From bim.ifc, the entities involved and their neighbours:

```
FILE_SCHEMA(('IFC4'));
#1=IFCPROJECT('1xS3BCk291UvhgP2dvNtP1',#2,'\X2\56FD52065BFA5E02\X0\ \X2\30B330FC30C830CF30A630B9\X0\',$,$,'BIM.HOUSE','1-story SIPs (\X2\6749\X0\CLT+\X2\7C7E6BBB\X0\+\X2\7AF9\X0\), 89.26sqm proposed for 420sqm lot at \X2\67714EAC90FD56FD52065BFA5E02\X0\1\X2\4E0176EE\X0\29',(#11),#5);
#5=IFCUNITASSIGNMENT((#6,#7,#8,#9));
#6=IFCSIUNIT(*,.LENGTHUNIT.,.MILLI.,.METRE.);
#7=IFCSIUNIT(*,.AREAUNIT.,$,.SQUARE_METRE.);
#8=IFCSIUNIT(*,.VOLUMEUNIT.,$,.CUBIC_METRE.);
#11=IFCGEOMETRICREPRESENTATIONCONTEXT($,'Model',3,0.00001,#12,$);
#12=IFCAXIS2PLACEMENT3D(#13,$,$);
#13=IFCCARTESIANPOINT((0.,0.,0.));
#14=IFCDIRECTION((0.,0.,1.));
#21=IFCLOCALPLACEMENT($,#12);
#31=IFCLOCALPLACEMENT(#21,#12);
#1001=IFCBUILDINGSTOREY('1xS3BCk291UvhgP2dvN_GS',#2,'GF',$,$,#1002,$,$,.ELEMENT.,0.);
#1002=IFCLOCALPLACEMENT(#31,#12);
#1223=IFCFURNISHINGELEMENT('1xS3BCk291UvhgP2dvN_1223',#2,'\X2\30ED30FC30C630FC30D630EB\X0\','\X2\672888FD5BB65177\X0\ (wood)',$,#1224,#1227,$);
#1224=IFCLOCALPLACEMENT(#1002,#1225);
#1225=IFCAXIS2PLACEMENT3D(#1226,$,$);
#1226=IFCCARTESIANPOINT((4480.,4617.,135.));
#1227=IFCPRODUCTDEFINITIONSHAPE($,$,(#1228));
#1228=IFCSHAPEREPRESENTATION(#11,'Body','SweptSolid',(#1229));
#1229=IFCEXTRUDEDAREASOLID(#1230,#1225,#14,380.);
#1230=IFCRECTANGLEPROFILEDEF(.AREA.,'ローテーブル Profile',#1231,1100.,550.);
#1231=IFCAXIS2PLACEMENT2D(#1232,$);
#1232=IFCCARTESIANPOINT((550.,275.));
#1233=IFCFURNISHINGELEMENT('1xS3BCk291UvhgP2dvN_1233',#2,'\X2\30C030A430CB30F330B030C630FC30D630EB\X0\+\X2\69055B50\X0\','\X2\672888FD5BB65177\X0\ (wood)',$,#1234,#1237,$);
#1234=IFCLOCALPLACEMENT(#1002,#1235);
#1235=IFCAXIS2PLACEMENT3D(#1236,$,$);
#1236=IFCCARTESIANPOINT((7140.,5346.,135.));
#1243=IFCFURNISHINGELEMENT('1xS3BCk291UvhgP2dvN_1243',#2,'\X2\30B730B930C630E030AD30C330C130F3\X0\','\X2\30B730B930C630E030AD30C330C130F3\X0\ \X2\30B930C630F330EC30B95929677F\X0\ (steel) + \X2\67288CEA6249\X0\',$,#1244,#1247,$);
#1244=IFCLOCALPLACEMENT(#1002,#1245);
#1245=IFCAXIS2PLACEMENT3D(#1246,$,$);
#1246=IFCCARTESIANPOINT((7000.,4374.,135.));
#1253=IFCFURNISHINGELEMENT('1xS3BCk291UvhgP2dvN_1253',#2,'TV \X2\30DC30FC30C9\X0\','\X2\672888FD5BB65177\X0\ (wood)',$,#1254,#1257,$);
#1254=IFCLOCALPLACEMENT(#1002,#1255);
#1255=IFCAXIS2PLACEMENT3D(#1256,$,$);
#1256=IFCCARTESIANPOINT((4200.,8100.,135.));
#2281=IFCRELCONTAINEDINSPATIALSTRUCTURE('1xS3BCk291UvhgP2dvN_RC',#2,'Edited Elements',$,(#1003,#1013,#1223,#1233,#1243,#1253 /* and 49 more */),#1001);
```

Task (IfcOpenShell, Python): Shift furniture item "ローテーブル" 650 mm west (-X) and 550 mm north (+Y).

```python
import ifcopenshell
import ifcopenshell.api.geometry
import ifcopenshell.util.placement
import ifcopenshell.util.unit

model = ifcopenshell.open("bim.ifc")
unit_scale = ifcopenshell.util.unit.calculate_unit_scale(model)

item = model.by_id(1223)
matrix = ifcopenshell.util.placement.get_local_placement(item.ObjectPlacement)
matrix[0, 3] -= 0.65 / unit_scale
matrix[1, 3] += 0.55 / unit_scale
ifcopenshell.api.geometry.edit_object_placement(model, product=item, matrix=matrix, is_si=False)

print(ifcopenshell.util.placement.get_local_placement(item.ObjectPlacement).round(3) + 0.0)

model.write("bim-out.ifc")
```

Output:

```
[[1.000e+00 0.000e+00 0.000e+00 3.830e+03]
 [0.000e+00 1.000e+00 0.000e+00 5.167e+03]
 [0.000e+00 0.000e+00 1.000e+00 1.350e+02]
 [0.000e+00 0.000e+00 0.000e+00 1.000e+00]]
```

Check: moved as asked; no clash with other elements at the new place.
